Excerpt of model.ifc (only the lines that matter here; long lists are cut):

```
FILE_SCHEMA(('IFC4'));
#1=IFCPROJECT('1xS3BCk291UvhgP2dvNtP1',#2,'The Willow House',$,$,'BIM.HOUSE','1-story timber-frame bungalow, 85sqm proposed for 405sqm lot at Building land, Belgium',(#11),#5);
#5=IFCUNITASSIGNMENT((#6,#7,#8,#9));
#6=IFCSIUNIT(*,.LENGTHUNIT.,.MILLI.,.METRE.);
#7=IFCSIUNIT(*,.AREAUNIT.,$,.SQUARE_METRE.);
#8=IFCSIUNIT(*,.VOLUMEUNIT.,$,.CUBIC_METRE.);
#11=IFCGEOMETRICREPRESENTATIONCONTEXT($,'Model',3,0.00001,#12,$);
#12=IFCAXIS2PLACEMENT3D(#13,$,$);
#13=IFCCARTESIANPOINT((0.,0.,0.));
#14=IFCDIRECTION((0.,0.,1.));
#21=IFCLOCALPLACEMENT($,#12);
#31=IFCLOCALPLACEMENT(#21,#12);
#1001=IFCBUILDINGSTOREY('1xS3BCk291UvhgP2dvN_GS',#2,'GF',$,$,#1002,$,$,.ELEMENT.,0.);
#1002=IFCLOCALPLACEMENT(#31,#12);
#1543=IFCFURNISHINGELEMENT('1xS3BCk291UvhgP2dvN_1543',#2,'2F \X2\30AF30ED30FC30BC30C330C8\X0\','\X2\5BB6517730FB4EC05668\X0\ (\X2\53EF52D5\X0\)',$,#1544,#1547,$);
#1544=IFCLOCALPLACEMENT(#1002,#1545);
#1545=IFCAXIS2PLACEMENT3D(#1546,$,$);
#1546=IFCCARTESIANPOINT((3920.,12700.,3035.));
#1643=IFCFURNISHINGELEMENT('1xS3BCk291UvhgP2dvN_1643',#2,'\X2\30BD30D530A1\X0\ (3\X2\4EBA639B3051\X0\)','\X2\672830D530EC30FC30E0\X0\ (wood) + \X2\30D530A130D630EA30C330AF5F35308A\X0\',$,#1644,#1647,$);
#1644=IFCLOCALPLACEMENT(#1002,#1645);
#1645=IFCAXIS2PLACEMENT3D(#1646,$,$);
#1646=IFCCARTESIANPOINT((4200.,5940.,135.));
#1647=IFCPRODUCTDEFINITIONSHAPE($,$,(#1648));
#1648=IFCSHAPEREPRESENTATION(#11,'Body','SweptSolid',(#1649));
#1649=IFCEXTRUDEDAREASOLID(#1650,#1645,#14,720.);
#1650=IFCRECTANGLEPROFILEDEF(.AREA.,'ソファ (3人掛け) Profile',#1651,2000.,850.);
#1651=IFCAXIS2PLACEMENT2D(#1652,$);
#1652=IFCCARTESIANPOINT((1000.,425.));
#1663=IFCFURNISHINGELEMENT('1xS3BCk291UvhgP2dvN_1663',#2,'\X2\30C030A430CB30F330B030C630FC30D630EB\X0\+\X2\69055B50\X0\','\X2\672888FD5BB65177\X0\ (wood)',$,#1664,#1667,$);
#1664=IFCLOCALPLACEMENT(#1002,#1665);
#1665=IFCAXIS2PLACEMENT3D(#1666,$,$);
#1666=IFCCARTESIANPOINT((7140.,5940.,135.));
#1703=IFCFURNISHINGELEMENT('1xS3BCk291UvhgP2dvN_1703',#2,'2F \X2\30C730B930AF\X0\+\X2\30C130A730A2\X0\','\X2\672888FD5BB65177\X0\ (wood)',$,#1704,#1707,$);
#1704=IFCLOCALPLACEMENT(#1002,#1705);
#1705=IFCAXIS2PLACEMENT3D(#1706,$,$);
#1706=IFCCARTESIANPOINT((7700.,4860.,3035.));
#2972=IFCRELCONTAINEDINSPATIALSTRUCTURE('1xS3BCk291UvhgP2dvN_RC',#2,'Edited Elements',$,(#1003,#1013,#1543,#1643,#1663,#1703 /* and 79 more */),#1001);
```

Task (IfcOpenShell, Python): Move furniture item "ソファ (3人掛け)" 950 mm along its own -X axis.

```python
import ifcopenshell
import ifcopenshell.api.geometry
import ifcopenshell.util.placement
import ifcopenshell.util.unit

model = ifcopenshell.open("model.ifc")
unit_scale = ifcopenshell.util.unit.calculate_unit_scale(model)

item = model.by_guid("1xS3BCk291UvhgP2dvN_1643")
matrix = ifcopenshell.util.placement.get_local_placement(item.ObjectPlacement)
matrix[:3, 3] -= matrix[:3, 0] * 0.95 / unit_scale
ifcopenshell.api.geometry.edit_object_placement(model, product=item, matrix=matrix, is_si=False)

print(ifcopenshell.util.placement.get_local_placement(item.ObjectPlacement).round(3) + 0.0)

model.write("model_v2.ifc")
```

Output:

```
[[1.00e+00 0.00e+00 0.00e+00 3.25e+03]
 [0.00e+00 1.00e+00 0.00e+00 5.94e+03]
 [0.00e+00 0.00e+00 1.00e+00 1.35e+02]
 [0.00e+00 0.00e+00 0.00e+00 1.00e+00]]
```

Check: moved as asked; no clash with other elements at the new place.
